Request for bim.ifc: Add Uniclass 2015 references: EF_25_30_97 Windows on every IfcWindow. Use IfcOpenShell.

First a look at what the model holds.

```python
import ifcopenshell

model = ifcopenshell.open("bim.ifc")
print(model.schema)
print("classifications:", [c.Name for c in model.by_type("IfcClassification")])
for ifc_class in ("IfcDoor", "IfcRoof", "IfcStair", "IfcWall", "IfcWindow"):
    print(ifc_class, len(model.by_type(ifc_class)))
```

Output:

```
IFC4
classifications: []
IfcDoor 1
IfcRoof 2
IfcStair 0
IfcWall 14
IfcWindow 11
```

```python
import ifcopenshell
import ifcopenshell.api.classification

model = ifcopenshell.open("bim.ifc")

system = ifcopenshell.api.classification.add_classification(model, classification="Uniclass 2015")

codes = {
    "IfcWindow": ("EF_25_30_97", "Windows"),
}
for ifc_class, (code, name) in codes.items():
    products = model.by_type(ifc_class)
    ifcopenshell.api.classification.add_reference(
        model, products=products, classification=system, identification=code, name=name
    )
    print(code, len(products))

model.write("bim_edited.ifc")
```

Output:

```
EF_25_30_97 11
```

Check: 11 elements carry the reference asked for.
